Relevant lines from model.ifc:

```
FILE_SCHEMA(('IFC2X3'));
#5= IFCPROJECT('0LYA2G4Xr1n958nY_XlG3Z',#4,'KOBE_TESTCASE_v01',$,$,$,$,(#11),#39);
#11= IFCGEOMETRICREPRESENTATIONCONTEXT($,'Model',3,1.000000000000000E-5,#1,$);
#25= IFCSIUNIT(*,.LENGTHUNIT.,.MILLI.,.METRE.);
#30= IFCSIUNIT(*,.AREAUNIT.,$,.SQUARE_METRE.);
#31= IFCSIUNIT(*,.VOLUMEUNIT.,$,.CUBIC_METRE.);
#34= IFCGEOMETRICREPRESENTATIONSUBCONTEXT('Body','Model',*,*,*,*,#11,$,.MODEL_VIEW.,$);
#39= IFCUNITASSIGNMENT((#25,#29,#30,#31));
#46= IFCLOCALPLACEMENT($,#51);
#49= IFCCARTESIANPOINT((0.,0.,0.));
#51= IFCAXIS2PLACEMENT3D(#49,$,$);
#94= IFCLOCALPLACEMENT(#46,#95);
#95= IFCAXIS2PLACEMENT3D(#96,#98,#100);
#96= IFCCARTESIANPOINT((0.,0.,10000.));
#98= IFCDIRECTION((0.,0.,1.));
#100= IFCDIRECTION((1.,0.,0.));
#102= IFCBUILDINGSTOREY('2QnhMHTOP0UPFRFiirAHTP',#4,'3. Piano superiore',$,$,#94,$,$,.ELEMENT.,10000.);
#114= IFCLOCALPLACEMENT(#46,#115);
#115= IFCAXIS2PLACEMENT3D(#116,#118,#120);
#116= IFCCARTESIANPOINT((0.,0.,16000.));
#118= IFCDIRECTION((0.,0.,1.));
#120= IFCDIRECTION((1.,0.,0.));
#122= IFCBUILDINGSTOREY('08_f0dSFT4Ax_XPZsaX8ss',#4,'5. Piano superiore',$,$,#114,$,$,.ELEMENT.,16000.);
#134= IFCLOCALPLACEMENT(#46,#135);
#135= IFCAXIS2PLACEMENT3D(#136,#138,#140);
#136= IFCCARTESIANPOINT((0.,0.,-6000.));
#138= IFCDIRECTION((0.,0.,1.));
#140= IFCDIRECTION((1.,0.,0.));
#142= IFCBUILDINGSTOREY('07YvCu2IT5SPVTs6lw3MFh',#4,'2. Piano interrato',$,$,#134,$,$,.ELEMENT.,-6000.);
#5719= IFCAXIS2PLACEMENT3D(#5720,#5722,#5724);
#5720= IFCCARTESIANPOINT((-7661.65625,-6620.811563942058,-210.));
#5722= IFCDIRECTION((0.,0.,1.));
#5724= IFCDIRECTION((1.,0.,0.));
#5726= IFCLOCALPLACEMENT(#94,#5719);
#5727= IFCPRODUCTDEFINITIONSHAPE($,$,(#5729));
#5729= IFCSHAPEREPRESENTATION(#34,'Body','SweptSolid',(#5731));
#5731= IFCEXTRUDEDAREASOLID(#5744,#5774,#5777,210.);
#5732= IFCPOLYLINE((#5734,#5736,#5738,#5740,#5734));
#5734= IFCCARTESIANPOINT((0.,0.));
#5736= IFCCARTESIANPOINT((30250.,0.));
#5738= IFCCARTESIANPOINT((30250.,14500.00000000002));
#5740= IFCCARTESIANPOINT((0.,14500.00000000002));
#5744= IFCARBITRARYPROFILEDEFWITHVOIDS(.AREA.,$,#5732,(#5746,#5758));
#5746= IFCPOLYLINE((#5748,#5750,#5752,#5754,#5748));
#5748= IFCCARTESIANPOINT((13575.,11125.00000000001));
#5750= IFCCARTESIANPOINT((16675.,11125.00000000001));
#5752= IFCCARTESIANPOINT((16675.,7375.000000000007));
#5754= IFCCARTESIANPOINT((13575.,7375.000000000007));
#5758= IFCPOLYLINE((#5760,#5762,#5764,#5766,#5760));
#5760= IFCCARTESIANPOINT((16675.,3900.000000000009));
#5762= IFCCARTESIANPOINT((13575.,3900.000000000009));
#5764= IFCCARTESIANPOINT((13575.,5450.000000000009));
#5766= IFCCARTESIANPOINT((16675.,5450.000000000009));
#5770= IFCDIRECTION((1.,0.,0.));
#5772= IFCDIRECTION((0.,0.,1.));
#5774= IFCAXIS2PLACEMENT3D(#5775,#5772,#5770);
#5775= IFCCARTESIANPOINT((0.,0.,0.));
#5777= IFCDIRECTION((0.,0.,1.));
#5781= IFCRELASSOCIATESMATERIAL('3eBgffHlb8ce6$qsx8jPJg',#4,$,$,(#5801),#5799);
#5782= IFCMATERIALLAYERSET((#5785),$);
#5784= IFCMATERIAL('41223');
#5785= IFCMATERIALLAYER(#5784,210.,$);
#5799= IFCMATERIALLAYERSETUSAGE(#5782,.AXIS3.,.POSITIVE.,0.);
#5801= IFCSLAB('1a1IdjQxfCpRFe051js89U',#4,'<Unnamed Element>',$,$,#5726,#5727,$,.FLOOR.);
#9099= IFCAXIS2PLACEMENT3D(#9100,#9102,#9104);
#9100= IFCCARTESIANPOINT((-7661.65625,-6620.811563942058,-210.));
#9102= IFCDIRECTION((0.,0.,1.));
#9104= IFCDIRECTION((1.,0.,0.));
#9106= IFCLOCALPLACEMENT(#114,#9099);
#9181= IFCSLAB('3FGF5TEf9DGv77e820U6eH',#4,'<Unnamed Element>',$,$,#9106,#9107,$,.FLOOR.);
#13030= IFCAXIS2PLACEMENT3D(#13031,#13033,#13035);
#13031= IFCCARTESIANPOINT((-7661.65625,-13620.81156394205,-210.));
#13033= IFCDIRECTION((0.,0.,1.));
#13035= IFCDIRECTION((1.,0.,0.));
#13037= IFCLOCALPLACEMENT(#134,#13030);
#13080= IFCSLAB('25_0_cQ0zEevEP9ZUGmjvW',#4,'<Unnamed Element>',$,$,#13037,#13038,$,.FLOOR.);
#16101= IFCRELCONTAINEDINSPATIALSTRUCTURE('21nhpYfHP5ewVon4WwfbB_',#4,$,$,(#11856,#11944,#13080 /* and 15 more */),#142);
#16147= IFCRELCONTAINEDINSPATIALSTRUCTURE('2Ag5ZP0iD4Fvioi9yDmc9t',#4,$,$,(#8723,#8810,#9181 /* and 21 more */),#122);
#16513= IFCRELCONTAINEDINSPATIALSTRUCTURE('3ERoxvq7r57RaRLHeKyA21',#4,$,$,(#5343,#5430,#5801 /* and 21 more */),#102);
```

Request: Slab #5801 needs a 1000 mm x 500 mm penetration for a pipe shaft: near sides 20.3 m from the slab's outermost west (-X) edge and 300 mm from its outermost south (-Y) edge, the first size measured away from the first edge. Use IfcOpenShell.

```python
import numpy as np
import ifcopenshell
import ifcopenshell.api.feature
import ifcopenshell.api.geometry
import ifcopenshell.api.root
import ifcopenshell.geom
import ifcopenshell.util.placement
import ifcopenshell.util.representation
import ifcopenshell.util.shape
import ifcopenshell.util.unit

model = ifcopenshell.open("model.ifc")
unit_scale = ifcopenshell.util.unit.calculate_unit_scale(model)
settings = ifcopenshell.geom.settings()


def volume(element):
    """Net volume in cubic metres, openings subtracted."""
    shape = ifcopenshell.geom.create_shape(settings, element)
    return ifcopenshell.util.shape.get_volume(shape.geometry)


slab = model.by_guid("1a1IdjQxfCpRFe051js89U")
before = volume(slab)

# Extent in the slab's own axes, in metres. The edges named are its -X and -Y sides.
slab_shape = ifcopenshell.geom.create_shape(settings, slab)
vertices = ifcopenshell.util.shape.get_vertices(slab_shape.geometry)
x_min, y_min, bottom = vertices.min(axis=0)
top = vertices[:, 2].max()

opening = ifcopenshell.api.root.create_entity(model, ifc_class="IfcOpeningElement", name="Pipe shaft opening")
context = ifcopenshell.util.representation.get_context(model, "Model", "Body", "MODEL_VIEW")
width, depth = 1, 0.5
outline = [(0.0, 0.0), (width, 0.0), (width, depth), (0.0, depth), (0.0, 0.0)]
# Overshoot both faces by 50 mm so the cut is clean.
shape = ifcopenshell.api.geometry.add_slab_representation(
    model, context=context, depth=top - bottom + 0.1, polyline=outline
)
ifcopenshell.api.geometry.assign_representation(model, product=opening, representation=shape)

matrix = ifcopenshell.util.placement.get_local_placement(slab.ObjectPlacement)
matrix[:, 3] = matrix @ np.append(np.array([x_min + 20.3, y_min + 0.3, bottom - 0.05]) / unit_scale, 1.0)
ifcopenshell.api.geometry.edit_object_placement(model, product=opening, matrix=matrix, is_si=False)
ifcopenshell.api.feature.add_feature(model, feature=opening, element=slab)

after = volume(slab)

print(f"slab volume {before:.3f} -> {after:.3f} m3")

model.write("model_rev.ifc")
```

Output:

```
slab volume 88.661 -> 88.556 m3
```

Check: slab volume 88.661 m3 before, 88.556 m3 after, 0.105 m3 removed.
